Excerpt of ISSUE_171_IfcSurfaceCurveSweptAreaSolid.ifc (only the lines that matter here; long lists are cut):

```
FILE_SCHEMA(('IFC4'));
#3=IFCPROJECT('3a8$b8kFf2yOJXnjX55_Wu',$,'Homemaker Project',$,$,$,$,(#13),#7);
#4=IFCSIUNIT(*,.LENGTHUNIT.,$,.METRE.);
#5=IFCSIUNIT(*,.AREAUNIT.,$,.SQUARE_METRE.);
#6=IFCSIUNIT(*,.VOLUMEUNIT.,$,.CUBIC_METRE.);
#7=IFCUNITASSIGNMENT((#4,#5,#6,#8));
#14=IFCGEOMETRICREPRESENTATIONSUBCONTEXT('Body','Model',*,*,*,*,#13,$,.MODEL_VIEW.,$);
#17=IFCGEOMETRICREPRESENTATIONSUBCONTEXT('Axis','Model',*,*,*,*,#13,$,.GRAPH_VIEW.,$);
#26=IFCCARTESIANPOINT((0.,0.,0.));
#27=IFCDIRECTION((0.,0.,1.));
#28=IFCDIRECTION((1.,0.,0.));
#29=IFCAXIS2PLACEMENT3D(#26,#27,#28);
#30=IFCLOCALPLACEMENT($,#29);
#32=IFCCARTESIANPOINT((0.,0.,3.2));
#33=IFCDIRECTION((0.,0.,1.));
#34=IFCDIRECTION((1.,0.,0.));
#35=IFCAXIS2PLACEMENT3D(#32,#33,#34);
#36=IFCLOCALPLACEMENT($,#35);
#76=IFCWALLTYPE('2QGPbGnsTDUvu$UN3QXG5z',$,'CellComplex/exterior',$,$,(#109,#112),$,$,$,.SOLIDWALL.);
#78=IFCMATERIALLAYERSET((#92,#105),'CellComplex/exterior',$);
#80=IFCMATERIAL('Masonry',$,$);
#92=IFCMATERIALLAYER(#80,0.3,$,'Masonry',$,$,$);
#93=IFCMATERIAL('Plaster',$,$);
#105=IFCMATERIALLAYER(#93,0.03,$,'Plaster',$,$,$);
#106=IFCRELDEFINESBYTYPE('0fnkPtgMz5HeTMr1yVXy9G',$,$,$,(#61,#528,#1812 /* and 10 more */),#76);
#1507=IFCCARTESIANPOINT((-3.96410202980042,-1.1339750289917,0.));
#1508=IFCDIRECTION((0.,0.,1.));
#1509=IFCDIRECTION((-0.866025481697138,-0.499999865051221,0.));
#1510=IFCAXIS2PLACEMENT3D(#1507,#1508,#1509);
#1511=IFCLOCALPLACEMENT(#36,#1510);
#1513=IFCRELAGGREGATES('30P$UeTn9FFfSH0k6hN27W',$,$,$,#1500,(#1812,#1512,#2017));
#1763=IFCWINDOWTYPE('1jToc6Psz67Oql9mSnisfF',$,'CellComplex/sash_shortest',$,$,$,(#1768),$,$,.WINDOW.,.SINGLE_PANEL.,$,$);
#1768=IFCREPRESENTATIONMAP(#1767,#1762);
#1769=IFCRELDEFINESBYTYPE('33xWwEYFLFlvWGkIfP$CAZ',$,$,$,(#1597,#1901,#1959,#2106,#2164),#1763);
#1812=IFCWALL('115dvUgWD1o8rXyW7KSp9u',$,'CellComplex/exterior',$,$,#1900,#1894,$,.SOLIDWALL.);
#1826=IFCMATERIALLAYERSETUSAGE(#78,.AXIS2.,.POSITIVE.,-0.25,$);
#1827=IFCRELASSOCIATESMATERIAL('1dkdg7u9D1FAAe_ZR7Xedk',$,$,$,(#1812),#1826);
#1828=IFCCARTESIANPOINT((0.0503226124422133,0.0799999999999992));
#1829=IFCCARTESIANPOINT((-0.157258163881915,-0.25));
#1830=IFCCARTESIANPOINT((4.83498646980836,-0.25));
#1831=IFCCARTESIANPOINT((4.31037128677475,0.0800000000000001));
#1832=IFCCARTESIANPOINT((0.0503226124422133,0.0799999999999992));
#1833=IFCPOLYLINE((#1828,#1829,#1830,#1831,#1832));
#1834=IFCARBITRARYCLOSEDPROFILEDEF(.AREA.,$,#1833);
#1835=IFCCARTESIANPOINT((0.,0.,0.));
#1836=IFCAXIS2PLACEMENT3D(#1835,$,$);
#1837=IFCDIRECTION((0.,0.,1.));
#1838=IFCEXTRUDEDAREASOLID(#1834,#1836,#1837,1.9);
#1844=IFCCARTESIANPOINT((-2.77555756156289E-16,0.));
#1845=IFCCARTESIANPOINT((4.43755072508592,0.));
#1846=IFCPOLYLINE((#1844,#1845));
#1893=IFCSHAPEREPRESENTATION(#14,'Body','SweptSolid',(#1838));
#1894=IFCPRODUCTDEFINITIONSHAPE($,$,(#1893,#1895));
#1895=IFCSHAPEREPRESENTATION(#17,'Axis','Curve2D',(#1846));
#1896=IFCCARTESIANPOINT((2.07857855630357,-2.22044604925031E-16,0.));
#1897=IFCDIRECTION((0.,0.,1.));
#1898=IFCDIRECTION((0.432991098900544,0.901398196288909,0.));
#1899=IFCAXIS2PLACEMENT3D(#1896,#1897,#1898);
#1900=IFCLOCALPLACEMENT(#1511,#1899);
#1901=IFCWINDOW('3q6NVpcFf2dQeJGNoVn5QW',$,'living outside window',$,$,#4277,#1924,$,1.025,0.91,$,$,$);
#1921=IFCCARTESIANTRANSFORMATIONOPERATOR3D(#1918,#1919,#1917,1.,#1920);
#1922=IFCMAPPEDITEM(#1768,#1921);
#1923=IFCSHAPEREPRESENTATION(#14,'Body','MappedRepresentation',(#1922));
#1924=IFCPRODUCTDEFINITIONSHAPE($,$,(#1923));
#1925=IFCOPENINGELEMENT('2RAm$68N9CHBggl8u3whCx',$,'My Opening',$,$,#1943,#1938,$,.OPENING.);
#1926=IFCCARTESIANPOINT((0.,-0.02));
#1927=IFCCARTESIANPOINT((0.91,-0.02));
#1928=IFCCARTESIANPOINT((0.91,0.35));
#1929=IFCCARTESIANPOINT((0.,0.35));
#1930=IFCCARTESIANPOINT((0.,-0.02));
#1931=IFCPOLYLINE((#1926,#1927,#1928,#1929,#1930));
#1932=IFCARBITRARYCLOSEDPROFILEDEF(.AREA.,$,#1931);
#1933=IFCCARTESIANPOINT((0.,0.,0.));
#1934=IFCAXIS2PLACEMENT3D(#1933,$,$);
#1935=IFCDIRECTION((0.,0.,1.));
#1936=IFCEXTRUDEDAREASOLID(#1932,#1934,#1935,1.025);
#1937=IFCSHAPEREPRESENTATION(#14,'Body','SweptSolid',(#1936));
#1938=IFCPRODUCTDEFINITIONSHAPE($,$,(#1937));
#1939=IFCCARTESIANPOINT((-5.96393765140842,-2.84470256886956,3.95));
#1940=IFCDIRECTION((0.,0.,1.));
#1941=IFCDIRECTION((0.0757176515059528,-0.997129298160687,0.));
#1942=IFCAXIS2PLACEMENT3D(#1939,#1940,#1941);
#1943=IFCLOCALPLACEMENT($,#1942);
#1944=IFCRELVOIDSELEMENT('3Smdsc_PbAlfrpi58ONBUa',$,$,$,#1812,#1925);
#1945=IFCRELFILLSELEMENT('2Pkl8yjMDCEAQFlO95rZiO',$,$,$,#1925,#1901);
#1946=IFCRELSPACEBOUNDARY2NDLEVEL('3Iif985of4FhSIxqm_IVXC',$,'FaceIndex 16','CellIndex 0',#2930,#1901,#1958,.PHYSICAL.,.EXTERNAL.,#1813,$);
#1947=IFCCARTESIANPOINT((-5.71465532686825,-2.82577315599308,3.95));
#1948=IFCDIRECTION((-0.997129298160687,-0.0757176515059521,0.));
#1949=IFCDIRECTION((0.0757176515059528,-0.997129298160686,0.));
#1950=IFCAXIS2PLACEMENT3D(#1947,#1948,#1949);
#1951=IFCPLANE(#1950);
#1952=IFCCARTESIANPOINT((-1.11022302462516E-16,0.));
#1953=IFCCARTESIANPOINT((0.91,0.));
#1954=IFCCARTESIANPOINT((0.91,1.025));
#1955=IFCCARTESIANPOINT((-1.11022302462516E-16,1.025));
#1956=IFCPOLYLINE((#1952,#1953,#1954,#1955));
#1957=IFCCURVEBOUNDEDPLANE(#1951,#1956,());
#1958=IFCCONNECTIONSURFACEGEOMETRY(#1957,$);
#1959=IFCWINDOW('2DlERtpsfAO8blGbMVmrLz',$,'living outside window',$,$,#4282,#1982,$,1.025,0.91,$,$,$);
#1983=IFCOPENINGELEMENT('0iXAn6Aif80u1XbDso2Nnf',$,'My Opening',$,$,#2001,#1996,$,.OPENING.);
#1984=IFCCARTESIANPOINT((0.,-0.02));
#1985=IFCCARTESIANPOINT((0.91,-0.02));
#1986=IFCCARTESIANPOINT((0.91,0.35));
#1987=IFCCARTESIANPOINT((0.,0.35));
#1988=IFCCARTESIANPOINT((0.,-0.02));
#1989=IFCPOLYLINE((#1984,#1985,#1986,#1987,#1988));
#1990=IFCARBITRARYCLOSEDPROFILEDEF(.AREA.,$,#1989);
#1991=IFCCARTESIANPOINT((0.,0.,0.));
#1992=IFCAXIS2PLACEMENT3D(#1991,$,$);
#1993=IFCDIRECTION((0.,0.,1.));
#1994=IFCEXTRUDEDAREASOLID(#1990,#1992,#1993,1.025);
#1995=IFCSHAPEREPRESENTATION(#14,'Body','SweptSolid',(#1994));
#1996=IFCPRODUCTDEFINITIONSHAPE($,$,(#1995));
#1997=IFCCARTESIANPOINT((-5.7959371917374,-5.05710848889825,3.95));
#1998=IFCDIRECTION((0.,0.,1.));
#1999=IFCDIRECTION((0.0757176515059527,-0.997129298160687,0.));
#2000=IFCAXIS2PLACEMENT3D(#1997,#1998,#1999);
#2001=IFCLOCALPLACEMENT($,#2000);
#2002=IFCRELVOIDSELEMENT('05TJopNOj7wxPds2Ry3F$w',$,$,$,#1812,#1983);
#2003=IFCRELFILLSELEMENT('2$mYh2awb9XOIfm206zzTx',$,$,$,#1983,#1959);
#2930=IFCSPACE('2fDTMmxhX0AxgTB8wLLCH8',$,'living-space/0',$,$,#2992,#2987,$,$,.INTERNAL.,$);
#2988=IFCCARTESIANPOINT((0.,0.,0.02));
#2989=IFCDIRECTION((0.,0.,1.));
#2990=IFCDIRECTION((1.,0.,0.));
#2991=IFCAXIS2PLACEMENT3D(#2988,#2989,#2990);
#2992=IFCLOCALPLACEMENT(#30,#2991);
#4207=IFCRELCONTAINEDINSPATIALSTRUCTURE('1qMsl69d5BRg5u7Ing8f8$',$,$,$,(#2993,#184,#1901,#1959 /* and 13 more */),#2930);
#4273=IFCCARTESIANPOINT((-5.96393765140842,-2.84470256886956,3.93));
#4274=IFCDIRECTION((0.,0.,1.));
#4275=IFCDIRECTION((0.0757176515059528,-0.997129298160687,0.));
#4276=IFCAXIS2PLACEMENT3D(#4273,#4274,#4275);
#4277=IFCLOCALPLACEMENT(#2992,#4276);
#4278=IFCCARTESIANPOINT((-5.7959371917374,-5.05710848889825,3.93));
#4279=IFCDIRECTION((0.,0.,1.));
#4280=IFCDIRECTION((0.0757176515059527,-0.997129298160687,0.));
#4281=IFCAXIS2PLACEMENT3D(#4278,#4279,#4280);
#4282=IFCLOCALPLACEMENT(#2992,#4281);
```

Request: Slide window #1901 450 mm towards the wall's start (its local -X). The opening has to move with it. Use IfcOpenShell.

```python
import numpy as np
import ifcopenshell
import ifcopenshell.api.geometry
import ifcopenshell.util.placement
import ifcopenshell.util.unit

model = ifcopenshell.open("ISSUE_171_IfcSurfaceCurveSweptAreaSolid.ifc")
unit_scale = ifcopenshell.util.unit.calculate_unit_scale(model)

window = model.by_guid("3q6NVpcFf2dQeJGNoVn5QW")
opening = window.FillsVoids[0].RelatingOpeningElement
wall = opening.VoidsElements[0].RelatingBuildingElement

wall_matrix = ifcopenshell.util.placement.get_local_placement(wall.ObjectPlacement)
shift = wall_matrix[:3, 0] * -0.45 / unit_scale
before = ifcopenshell.util.placement.get_local_placement(window.ObjectPlacement)[:3, 3].copy()

# The window is not placed relative to its opening, so move both.
for product in (opening, window):
    matrix = ifcopenshell.util.placement.get_local_placement(product.ObjectPlacement)
    matrix[:3, 3] += shift
    ifcopenshell.api.geometry.edit_object_placement(model, product=product, matrix=matrix, is_si=False)

# Space boundary surfaces are stored in each space's coordinates; move them too.
for rel in window.ProvidesBoundaries:
    if not rel.ConnectionGeometry:
        continue
    surface = rel.ConnectionGeometry.SurfaceOnRelatingElement.BasisSurface
    space_matrix = ifcopenshell.util.placement.get_local_placement(rel.RelatingSpace.ObjectPlacement)
    point = np.array(surface.Position.Location.Coordinates) + space_matrix[:3, :3].T @ shift
    surface.Position = model.createIfcAxis2Placement3D(
        model.createIfcCartesianPoint(point.tolist()), surface.Position.Axis, surface.Position.RefDirection
    )

after = ifcopenshell.util.placement.get_local_placement(window.ObjectPlacement)[:3, 3]
print("window moved by", (after - before).round(3) + 0.0)

model.write("ISSUE_171_IfcSurfaceCurveSweptAreaSolid_edited.ifc")
```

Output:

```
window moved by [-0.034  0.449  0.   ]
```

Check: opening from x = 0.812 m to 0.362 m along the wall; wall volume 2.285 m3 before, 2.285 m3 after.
